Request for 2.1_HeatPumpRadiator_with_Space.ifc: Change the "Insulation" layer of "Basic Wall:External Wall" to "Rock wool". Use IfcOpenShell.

First a look at what the model holds.

```python
import ifcopenshell
import ifcopenshell.util.element

model = ifcopenshell.open("2.1_HeatPumpRadiator_with_Space.ifc")
print(model.schema)
for layer_set in model.by_type("IfcMaterialLayerSet"):
    if layer_set.LayerSetName == "Basic Wall:External Wall":
        for layer in layer_set.MaterialLayers:
            print(layer.id(), layer.Material and layer.Material.Name, layer.LayerThickness, sep=" | ")
        print(len(ifcopenshell.util.element.get_elements_by_material(model, layer_set)), "elements and types use it")
print(sorted(m.Name for m in model.by_type("IfcMaterial") if m.Name)[:60])
```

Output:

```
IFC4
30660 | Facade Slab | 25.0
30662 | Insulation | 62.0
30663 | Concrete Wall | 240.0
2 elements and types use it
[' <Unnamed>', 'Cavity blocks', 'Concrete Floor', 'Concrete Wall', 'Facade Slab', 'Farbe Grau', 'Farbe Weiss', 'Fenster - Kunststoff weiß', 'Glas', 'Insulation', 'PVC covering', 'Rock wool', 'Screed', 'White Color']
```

```python
import ifcopenshell
import ifcopenshell.api.material

model = ifcopenshell.open("2.1_HeatPumpRadiator_with_Space.ifc")

layer_set = next(s for s in model.by_type("IfcMaterialLayerSet") if s.LayerSetName == "Basic Wall:External Wall")
layer = next(l for l in layer_set.MaterialLayers if l.Material and l.Material.Name == "Insulation")
material = next(m for m in model.by_type("IfcMaterial") if m.Name == "Rock wool")

# Point this one layer at the other material; renaming the old one would change it everywhere.
ifcopenshell.api.material.edit_layer(model, layer=layer, attributes={}, material=material)

print([l.Material.Name if l.Material else None for l in layer_set.MaterialLayers])

model.write("2.1_HeatPumpRadiator_with_Space-out.ifc")
```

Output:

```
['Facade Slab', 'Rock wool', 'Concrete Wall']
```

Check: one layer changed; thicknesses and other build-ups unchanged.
